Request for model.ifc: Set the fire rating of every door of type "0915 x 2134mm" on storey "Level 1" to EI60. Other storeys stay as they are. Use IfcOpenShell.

First a look at what the model holds.

```python
import ifcopenshell
import ifcopenshell.util.element

model = ifcopenshell.open("model.ifc")
print(model.schema)
storey = next(s for s in model.by_type("IfcBuildingStorey") if s.Name == "Level 1")
doors = [e for e in ifcopenshell.util.element.get_decomposition(storey) if e.is_a("IfcDoor")]
seen = {}
for e in doors:
    element_type = ifcopenshell.util.element.get_type(e)
    key = (element_type.Name if element_type != e and element_type else None, ifcopenshell.util.element.get_pset(e, "Pset_DoorCommon", "FireRating"))
    seen[key] = seen.get(key, 0) + 1
for (name, value), count in sorted(seen.items(), key=str):
    print(count, "x", name, "|", value)
```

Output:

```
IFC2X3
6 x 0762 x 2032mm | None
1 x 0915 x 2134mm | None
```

```python
import ifcopenshell
import ifcopenshell.api.pset
import ifcopenshell.util.element

model = ifcopenshell.open("model.ifc")

storey = next(s for s in model.by_type("IfcBuildingStorey") if s.Name == "Level 1")
doors = [e for e in ifcopenshell.util.element.get_decomposition(storey) if e.is_a("IfcDoor")]

count = 0
for e in doors:
    element_type = ifcopenshell.util.element.get_type(e)
    if element_type in (None, e) or element_type.Name != "0915 x 2134mm":
        continue
    # add_pset returns the element's existing set when there is one.
    pset = ifcopenshell.api.pset.add_pset(model, product=e, name="Pset_DoorCommon")
    ifcopenshell.api.pset.edit_pset(model, pset=pset, properties={"FireRating": "EI60"})
    count += 1

print(count, "doors updated")

model.write("model_v2.ifc")
```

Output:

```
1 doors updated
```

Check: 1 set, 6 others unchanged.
